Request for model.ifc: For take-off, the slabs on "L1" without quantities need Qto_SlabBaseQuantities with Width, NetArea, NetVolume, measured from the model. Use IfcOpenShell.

First a look at what the model holds.

```python
import ifcopenshell
import ifcopenshell.util.element
import ifcopenshell.util.unit

model = ifcopenshell.open("model.ifc")
print(model.schema)
for unit_type in ("LENGTHUNIT", "AREAUNIT", "VOLUMEUNIT"):
    print(unit_type, ifcopenshell.util.unit.calculate_unit_scale(model, unit_type))
storey = next(s for s in model.by_type("IfcBuildingStorey") if s.Name == "L1")
slabs = [e for e in ifcopenshell.util.element.get_decomposition(storey) if e.is_a("IfcSlab")]
for e in sorted(slabs, key=lambda e: e.id()):
    print(e.id(), e.is_a(), e.Name, list(ifcopenshell.util.element.get_psets(e, qtos_only=True)), sep=" | ")
```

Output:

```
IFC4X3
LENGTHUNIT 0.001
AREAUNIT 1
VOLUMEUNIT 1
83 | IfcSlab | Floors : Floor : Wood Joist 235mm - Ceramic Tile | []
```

```python
import ifcopenshell
import ifcopenshell.api.pset
import ifcopenshell.geom
import ifcopenshell.util.element
import ifcopenshell.util.shape
import ifcopenshell.util.unit

model = ifcopenshell.open("model.ifc")
unit_scale = ifcopenshell.util.unit.calculate_unit_scale(model)
area_scale = ifcopenshell.util.unit.calculate_unit_scale(model, "AREAUNIT")
volume_scale = ifcopenshell.util.unit.calculate_unit_scale(model, "VOLUMEUNIT")
settings = ifcopenshell.geom.settings()

storey = next(s for s in model.by_type("IfcBuildingStorey") if s.Name == "L1")
slabs = [e for e in ifcopenshell.util.element.get_decomposition(storey) if e.is_a("IfcSlab")]

for e in sorted(slabs, key=lambda e: e.id()):
    if ifcopenshell.util.element.get_psets(e, qtos_only=True, should_inherit=False):
        continue
    # Geometry comes back in metres, in the element's own axes.
    shape = ifcopenshell.geom.create_shape(settings, e)
    values = {
        "Width": ifcopenshell.util.shape.get_z(shape.geometry) / unit_scale,
        "NetArea": ifcopenshell.util.shape.get_footprint_area(shape.geometry) / area_scale,
        "NetVolume": ifcopenshell.util.shape.get_volume(shape.geometry) / volume_scale,
    }
    qto = ifcopenshell.api.pset.add_qto(model, product=e, name="Qto_SlabBaseQuantities")
    ifcopenshell.api.pset.edit_qto(model, qto=qto, properties=values)
    print(e.id(), {k: round(v, 3) for k, v in values.items()})

model.write("model_v2.ifc")
```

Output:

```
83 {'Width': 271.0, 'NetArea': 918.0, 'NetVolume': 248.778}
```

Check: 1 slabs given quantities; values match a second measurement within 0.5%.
